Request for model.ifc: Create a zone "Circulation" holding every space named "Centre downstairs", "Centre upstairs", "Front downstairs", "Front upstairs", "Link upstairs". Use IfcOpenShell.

First a look at what the model holds.

```python
import ifcopenshell

model = ifcopenshell.open("model.ifc")
print(model.schema)
seen = {}
for space in model.by_type("IfcSpace"):
    seen[space.Name] = seen.get(space.Name, 0) + 1
for name, count in sorted(seen.items(), key=str):
    print(count, "x", name)
print("zones:", [z.Name for z in model.by_type("IfcZone")][:20])
```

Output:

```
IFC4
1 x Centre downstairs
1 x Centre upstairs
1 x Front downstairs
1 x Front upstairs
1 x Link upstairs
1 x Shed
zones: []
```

```python
import ifcopenshell
import ifcopenshell.api.group
import ifcopenshell.api.root

model = ifcopenshell.open("model.ifc")

names = {"Centre downstairs", "Centre upstairs", "Front downstairs", "Front upstairs", "Link upstairs"}
spaces = [s for s in model.by_type("IfcSpace") if s.Name in names]

zone = ifcopenshell.api.root.create_entity(model, ifc_class="IfcZone", name="Circulation")
ifcopenshell.api.group.assign_group(model, products=spaces, group=zone)
print(len(spaces), "spaces in", zone.Name)

model.write("model-out.ifc")
```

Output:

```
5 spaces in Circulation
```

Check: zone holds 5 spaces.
